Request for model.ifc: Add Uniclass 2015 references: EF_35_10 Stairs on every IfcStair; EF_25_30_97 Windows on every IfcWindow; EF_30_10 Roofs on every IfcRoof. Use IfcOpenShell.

First a look at what the model holds.

```python
import ifcopenshell

model = ifcopenshell.open("model.ifc")
print(model.schema)
print("classifications:", [c.Name for c in model.by_type("IfcClassification")])
for ifc_class in ("IfcDoor", "IfcRoof", "IfcStair", "IfcWall", "IfcWindow"):
    print(ifc_class, len(model.by_type(ifc_class)))
```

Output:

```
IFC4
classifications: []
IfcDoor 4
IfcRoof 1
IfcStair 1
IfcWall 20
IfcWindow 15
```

```python
import ifcopenshell
import ifcopenshell.api.classification

model = ifcopenshell.open("model.ifc")

system = ifcopenshell.api.classification.add_classification(model, classification="Uniclass 2015")

codes = {
    "IfcStair": ("EF_35_10", "Stairs"),
    "IfcWindow": ("EF_25_30_97", "Windows"),
    "IfcRoof": ("EF_30_10", "Roofs"),
}
for ifc_class, (code, name) in codes.items():
    products = model.by_type(ifc_class)
    ifcopenshell.api.classification.add_reference(
        model, products=products, classification=system, identification=code, name=name
    )
    print(code, len(products))

model.write("model_updated.ifc")
```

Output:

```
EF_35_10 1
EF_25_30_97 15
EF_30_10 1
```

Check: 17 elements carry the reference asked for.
